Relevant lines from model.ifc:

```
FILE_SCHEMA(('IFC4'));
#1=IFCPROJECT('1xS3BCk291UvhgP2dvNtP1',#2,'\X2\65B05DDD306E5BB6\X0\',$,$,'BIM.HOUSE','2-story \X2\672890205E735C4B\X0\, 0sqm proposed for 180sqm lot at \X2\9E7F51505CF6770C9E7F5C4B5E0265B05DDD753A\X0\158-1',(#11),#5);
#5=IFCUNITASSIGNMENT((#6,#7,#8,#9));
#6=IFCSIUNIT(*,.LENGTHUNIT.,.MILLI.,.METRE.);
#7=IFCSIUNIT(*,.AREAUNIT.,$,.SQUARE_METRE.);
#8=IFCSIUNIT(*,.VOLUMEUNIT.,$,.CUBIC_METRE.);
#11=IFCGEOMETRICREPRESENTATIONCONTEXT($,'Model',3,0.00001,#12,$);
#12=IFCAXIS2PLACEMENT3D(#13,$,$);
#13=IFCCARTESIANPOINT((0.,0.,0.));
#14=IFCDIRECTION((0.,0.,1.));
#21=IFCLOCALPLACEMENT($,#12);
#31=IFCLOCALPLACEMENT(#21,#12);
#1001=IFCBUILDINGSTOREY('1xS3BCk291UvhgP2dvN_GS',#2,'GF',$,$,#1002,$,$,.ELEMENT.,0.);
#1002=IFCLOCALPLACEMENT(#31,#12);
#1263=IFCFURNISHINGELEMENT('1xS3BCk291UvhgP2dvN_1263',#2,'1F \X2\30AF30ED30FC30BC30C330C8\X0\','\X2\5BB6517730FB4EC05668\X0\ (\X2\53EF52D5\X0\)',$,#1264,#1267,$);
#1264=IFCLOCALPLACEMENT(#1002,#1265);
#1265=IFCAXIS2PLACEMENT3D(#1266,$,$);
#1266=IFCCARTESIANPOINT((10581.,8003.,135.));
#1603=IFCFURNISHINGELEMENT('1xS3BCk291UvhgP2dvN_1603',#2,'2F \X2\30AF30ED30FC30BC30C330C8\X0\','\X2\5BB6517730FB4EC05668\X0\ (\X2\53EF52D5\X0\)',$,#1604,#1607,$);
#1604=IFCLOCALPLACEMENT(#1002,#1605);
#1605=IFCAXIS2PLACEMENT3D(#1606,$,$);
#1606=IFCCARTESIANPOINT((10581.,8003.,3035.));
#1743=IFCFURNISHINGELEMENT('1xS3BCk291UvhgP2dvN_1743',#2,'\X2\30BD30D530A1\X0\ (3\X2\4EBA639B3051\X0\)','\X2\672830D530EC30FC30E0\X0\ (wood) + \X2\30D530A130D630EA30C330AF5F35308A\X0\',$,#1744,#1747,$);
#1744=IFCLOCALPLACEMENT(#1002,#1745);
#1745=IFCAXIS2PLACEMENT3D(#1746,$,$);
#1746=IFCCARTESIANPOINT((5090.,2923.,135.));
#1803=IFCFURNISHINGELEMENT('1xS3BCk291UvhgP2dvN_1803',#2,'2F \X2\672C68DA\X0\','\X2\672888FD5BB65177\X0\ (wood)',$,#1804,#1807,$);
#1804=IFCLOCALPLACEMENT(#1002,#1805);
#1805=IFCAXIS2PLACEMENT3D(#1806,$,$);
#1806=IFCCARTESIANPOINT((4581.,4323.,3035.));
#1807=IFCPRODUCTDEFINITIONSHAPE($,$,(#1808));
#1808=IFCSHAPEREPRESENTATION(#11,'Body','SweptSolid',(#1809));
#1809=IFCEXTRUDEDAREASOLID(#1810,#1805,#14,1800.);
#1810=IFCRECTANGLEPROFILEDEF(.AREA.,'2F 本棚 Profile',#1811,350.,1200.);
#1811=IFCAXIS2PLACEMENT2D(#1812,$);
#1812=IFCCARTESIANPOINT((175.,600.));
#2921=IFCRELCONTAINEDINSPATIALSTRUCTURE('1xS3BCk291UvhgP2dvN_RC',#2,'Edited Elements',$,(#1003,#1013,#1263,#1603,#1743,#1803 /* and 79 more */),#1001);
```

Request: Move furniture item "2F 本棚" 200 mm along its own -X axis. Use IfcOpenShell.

```python
import ifcopenshell
import ifcopenshell.api.geometry
import ifcopenshell.util.placement

model = ifcopenshell.open("model.ifc")

item = model.by_guid("1xS3BCk291UvhgP2dvN_1803")
matrix = ifcopenshell.util.placement.get_local_placement(item.ObjectPlacement)
matrix[:3, 3] -= matrix[:3, 0] * 200.0
ifcopenshell.api.geometry.edit_object_placement(model, product=item, matrix=matrix, is_si=False)

print(ifcopenshell.util.placement.get_local_placement(item.ObjectPlacement).round(3) + 0.0)

model.write("model_updated.ifc")
```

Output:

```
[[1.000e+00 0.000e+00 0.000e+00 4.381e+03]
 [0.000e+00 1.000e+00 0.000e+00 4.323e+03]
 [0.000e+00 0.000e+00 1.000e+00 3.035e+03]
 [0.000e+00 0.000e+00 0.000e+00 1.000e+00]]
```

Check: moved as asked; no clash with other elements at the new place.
